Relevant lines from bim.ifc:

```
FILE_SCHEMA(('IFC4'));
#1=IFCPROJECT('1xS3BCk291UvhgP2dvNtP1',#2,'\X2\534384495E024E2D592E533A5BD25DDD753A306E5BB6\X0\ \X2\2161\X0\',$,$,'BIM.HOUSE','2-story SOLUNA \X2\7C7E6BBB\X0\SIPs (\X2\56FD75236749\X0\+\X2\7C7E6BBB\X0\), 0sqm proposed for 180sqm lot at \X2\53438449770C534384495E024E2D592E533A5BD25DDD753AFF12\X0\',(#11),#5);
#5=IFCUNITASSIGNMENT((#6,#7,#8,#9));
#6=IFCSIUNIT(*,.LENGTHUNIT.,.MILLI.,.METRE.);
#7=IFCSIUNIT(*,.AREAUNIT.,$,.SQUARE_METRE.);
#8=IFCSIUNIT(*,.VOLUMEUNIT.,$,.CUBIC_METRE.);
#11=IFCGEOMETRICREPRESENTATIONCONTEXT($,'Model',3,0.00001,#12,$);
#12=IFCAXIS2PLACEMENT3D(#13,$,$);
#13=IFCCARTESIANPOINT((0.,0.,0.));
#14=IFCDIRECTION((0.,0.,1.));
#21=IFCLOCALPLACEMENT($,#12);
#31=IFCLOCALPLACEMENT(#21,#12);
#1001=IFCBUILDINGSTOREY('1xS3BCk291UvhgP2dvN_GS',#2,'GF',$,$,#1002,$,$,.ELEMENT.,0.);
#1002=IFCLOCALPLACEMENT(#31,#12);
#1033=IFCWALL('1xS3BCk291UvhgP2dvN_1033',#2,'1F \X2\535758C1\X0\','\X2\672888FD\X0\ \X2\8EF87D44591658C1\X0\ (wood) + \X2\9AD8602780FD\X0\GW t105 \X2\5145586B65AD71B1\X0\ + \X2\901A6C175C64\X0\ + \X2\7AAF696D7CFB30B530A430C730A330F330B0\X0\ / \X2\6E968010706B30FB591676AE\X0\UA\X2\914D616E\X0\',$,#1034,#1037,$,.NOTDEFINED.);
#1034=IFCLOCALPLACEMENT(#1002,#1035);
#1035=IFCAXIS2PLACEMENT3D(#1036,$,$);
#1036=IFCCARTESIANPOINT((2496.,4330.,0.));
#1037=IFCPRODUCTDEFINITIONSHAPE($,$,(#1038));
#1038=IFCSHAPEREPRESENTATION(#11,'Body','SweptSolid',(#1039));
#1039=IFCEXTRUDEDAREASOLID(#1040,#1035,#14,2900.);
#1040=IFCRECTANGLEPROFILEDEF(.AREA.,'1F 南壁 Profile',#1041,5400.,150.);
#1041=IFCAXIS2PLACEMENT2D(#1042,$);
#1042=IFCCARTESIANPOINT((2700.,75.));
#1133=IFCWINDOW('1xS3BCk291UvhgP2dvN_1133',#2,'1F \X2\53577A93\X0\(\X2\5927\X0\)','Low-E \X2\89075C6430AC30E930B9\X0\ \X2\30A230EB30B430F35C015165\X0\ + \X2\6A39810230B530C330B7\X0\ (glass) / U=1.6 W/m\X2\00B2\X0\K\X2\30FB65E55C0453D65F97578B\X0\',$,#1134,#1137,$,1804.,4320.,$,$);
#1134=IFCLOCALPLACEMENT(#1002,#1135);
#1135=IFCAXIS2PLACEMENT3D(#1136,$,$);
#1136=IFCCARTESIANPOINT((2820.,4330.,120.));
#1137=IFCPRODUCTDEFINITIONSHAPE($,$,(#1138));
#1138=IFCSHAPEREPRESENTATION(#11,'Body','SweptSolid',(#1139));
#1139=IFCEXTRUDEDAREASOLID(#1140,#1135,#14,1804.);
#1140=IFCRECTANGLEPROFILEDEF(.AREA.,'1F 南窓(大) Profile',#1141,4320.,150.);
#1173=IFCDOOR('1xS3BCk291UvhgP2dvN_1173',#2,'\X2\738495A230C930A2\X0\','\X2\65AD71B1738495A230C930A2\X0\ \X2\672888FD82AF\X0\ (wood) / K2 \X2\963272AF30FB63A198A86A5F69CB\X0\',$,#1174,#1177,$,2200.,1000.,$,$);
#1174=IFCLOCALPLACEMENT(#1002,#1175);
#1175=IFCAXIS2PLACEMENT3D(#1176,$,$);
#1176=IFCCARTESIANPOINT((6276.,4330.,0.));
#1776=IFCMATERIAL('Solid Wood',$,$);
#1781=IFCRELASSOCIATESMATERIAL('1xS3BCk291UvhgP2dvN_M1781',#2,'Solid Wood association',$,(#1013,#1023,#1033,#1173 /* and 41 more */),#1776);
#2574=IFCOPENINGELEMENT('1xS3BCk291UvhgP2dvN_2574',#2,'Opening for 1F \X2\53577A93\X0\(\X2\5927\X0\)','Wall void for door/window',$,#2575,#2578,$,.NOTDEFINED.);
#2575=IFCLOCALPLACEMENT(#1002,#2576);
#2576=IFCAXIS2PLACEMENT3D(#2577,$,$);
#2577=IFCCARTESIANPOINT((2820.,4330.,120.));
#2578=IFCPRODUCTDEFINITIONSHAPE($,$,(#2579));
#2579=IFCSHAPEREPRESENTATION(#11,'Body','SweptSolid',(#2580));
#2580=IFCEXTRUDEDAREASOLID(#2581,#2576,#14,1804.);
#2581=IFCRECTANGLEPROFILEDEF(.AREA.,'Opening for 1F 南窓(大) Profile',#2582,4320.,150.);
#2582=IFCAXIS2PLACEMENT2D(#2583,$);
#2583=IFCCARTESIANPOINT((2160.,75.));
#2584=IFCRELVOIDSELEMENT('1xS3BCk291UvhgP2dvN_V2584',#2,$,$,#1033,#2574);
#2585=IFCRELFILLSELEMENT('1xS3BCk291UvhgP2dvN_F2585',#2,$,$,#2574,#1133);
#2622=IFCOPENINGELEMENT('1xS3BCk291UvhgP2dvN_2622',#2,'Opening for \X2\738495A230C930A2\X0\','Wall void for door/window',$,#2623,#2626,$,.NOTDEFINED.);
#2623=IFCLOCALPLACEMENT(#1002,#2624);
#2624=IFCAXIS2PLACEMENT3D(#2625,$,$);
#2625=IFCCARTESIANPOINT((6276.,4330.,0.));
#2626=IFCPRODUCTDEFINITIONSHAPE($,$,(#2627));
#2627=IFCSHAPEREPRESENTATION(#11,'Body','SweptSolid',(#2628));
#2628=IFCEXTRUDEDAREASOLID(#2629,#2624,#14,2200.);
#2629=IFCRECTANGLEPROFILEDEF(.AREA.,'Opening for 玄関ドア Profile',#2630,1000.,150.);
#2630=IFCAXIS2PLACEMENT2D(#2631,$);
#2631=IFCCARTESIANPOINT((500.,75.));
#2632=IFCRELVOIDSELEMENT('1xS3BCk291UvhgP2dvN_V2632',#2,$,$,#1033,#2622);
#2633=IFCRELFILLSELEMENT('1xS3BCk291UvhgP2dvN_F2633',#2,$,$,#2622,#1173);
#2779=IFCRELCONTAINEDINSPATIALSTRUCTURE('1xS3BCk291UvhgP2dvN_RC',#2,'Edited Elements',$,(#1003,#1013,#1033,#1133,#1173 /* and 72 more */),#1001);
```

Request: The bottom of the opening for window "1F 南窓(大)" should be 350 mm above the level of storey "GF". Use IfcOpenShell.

```python
import numpy as np
import ifcopenshell
import ifcopenshell.api.geometry
import ifcopenshell.geom
import ifcopenshell.util.element
import ifcopenshell.util.placement
import ifcopenshell.util.shape
import ifcopenshell.util.unit

model = ifcopenshell.open("bim.ifc")
unit_scale = ifcopenshell.util.unit.calculate_unit_scale(model)

window = model.by_guid("1xS3BCk291UvhgP2dvN_1133")
opening = window.FillsVoids[0].RelatingOpeningElement
storey = ifcopenshell.util.element.get_container(window, ifc_class="IfcBuildingStorey")
level = ifcopenshell.util.placement.get_local_placement(storey.ObjectPlacement)[2, 3]

# The opening's origin need not be at the sill, so measure its lowest point.
shape = ifcopenshell.geom.create_shape(ifcopenshell.geom.settings(), opening)
bottom = ifcopenshell.util.shape.get_shape_bottom_elevation(shape, shape.geometry) / unit_scale
dz = level + 350.0 - bottom

shift = np.array([0.0, 0.0, dz])
# The window is not placed relative to its opening, so move both.
for product in (opening, window):
    matrix = ifcopenshell.util.placement.get_local_placement(product.ObjectPlacement)
    matrix[:3, 3] += shift
    ifcopenshell.api.geometry.edit_object_placement(model, product=product, matrix=matrix, is_si=False)

print(f"moved by {dz * unit_scale:+.3f} m")

model.write("bim-out.ifc")
```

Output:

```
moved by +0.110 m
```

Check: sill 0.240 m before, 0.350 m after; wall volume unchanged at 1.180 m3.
